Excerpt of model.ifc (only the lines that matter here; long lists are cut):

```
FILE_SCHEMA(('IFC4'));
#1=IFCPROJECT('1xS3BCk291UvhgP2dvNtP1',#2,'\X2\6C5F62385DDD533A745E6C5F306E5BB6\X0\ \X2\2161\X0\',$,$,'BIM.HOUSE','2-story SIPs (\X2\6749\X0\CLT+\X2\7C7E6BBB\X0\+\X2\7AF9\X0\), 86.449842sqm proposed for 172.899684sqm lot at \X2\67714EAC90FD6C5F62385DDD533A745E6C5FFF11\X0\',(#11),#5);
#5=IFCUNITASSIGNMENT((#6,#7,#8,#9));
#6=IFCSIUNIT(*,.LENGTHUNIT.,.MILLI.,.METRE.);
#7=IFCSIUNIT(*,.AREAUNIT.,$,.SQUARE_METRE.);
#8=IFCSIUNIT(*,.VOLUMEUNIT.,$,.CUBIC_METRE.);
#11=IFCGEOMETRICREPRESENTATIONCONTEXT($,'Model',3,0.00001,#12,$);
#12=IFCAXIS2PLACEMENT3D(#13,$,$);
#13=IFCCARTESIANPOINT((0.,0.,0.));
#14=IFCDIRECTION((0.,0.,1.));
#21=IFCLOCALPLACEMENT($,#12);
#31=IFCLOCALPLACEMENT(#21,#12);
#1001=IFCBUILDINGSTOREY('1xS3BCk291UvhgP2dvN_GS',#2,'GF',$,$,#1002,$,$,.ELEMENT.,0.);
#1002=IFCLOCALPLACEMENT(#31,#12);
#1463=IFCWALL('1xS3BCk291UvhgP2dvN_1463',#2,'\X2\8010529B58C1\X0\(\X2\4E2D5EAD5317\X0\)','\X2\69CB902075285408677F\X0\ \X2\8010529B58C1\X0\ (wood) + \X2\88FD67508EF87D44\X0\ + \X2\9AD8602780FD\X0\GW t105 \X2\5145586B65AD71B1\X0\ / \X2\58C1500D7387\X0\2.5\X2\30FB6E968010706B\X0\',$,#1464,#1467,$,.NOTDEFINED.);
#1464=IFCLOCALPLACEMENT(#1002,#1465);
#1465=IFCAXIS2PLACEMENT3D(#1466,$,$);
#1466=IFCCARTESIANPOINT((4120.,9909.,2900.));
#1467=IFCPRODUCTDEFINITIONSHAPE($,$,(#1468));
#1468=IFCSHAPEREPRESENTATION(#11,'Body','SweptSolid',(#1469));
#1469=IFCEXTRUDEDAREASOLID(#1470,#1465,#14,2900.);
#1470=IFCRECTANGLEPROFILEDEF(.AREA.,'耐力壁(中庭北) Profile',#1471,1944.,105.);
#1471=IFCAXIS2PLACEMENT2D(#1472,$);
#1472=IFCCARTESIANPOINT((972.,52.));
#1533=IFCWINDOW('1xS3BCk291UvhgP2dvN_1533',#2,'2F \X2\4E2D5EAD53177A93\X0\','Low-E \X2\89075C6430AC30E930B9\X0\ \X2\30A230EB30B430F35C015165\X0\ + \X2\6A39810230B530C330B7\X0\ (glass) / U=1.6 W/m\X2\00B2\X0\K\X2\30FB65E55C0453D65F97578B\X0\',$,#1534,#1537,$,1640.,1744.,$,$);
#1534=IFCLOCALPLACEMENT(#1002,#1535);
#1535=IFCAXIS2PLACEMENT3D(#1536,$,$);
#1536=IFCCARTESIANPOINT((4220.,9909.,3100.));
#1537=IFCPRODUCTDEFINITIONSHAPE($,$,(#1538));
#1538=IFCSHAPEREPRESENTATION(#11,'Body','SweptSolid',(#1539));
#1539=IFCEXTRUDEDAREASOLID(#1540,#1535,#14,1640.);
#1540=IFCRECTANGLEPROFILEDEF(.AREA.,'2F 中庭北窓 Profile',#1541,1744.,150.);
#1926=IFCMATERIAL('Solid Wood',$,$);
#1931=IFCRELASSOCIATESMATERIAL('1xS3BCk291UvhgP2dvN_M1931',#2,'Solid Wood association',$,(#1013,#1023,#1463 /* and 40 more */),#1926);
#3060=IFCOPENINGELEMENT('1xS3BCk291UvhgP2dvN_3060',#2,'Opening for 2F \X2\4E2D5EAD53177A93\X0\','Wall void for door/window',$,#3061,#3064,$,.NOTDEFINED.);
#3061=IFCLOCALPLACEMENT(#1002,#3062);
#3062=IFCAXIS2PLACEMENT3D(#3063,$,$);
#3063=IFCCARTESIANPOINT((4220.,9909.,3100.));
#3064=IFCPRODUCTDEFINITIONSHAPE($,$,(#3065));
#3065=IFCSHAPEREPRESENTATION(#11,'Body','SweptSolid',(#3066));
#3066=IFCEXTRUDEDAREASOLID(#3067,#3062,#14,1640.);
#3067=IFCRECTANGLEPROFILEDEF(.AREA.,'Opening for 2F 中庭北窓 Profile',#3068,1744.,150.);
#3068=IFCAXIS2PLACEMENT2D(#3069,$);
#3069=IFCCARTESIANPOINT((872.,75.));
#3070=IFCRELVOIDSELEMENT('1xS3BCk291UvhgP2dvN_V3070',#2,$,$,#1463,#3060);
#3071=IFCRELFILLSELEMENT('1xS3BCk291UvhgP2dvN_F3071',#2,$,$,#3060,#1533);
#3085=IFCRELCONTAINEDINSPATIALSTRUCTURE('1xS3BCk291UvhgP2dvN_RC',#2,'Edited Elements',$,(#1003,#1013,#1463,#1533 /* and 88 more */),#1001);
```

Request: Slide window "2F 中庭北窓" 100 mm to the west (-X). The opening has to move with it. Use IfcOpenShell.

```python
import ifcopenshell
import ifcopenshell.api.geometry
import ifcopenshell.util.placement
import ifcopenshell.util.unit

model = ifcopenshell.open("model.ifc")
unit_scale = ifcopenshell.util.unit.calculate_unit_scale(model)

window = model.by_guid("1xS3BCk291UvhgP2dvN_1533")
opening = window.FillsVoids[0].RelatingOpeningElement
wall = opening.VoidsElements[0].RelatingBuildingElement

wall_matrix = ifcopenshell.util.placement.get_local_placement(wall.ObjectPlacement)
shift = wall_matrix[:3, 0] * -0.1 / unit_scale
before = ifcopenshell.util.placement.get_local_placement(window.ObjectPlacement)[:3, 3].copy()

# The window is not placed relative to its opening, so move both.
for product in (opening, window):
    matrix = ifcopenshell.util.placement.get_local_placement(product.ObjectPlacement)
    matrix[:3, 3] += shift
    ifcopenshell.api.geometry.edit_object_placement(model, product=product, matrix=matrix, is_si=False)

after = ifcopenshell.util.placement.get_local_placement(window.ObjectPlacement)[:3, 3]
print("window moved by", (after - before).round(3) + 0.0)

model.write("model_v2.ifc")
```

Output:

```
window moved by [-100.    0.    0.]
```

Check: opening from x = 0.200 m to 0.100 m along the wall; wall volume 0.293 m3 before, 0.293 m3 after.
